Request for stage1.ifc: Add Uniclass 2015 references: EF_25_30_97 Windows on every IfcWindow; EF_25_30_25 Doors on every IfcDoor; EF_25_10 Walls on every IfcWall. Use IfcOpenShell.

First a look at what the model holds.

```python
import ifcopenshell

model = ifcopenshell.open("stage1.ifc")
print(model.schema)
print("classifications:", [c.Name for c in model.by_type("IfcClassification")])
for ifc_class in ("IfcDoor", "IfcRoof", "IfcStair", "IfcWall", "IfcWindow"):
    print(ifc_class, len(model.by_type(ifc_class)))
```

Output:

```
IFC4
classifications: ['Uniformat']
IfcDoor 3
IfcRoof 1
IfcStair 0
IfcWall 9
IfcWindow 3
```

```python
import ifcopenshell
import ifcopenshell.api.classification

model = ifcopenshell.open("stage1.ifc")

system = ifcopenshell.api.classification.add_classification(model, classification="Uniclass 2015")

codes = {
    "IfcWindow": ("EF_25_30_97", "Windows"),
    "IfcDoor": ("EF_25_30_25", "Doors"),
    "IfcWall": ("EF_25_10", "Walls"),
}
for ifc_class, (code, name) in codes.items():
    products = model.by_type(ifc_class)
    ifcopenshell.api.classification.add_reference(
        model, products=products, classification=system, identification=code, name=name
    )
    print(code, len(products))

model.write("stage1_rev.ifc")
```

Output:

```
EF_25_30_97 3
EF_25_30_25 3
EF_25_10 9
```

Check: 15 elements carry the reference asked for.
